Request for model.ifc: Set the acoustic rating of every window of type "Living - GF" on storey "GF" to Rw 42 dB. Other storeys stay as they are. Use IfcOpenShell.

First a look at what the model holds.

```python
import ifcopenshell
import ifcopenshell.util.element

model = ifcopenshell.open("model.ifc")
print(model.schema)
storey = next(s for s in model.by_type("IfcBuildingStorey") if s.Name == "GF")
windows = [e for e in ifcopenshell.util.element.get_decomposition(storey) if e.is_a("IfcWindow")]
seen = {}
for e in windows:
    element_type = ifcopenshell.util.element.get_type(e)
    key = (element_type.Name if element_type != e and element_type else None, ifcopenshell.util.element.get_pset(e, "Pset_WindowCommon", "AcousticRating"))
    seen[key] = seen.get(key, 0) + 1
for (name, value), count in sorted(seen.items(), key=str):
    print(count, "x", name, "|", value)
```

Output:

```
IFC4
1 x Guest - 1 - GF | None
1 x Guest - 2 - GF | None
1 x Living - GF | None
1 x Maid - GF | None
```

```python
import ifcopenshell
import ifcopenshell.api.pset
import ifcopenshell.util.element

model = ifcopenshell.open("model.ifc")

storey = next(s for s in model.by_type("IfcBuildingStorey") if s.Name == "GF")
windows = [e for e in ifcopenshell.util.element.get_decomposition(storey) if e.is_a("IfcWindow")]

count = 0
for e in windows:
    element_type = ifcopenshell.util.element.get_type(e)
    if element_type in (None, e) or element_type.Name != "Living - GF":
        continue
    # add_pset returns the element's existing set when there is one.
    pset = ifcopenshell.api.pset.add_pset(model, product=e, name="Pset_WindowCommon")
    ifcopenshell.api.pset.edit_pset(model, pset=pset, properties={"AcousticRating": "Rw 42 dB"})
    count += 1

print(count, "windows updated")

model.write("model_edited.ifc")
```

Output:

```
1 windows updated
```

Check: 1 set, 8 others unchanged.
